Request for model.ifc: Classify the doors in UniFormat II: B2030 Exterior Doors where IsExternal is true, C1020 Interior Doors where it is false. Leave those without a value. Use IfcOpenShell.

First a look at what the model holds.

```python
import ifcopenshell
import ifcopenshell.util.element

model = ifcopenshell.open("model.ifc")
print(model.schema)
print("classifications:", [c.Name for c in model.by_type("IfcClassification")])
values = [ifcopenshell.util.element.get_pset(e, "Pset_DoorCommon", "IsExternal") for e in model.by_type("IfcDoor")]
for value in (True, False, None):
    print("IsExternal", value, values.count(value))
```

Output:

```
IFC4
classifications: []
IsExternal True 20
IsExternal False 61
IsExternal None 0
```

```python
import ifcopenshell
import ifcopenshell.api.classification
import ifcopenshell.util.element

model = ifcopenshell.open("model.ifc")

system = ifcopenshell.api.classification.add_classification(model, classification="UniFormat II")

doors = model.by_type("IfcDoor")
external = {e: ifcopenshell.util.element.get_pset(e, "Pset_DoorCommon", "IsExternal") for e in doors}
for flag, code, name in ((True, "B2030", "Exterior Doors"), (False, "C1020", "Interior Doors")):
    products = [e for e in doors if external[e] is flag]
    ifcopenshell.api.classification.add_reference(
        model, products=products, classification=system, identification=code, name=name
    )
    print(code, len(products))

model.write("model_updated.ifc")
```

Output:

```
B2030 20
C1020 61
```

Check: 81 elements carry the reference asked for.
